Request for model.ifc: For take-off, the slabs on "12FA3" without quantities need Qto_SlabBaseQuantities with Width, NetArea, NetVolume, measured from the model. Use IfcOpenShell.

First a look at what the model holds.

```python
import ifcopenshell
import ifcopenshell.util.element
import ifcopenshell.util.unit

model = ifcopenshell.open("model.ifc")
print(model.schema)
for unit_type in ("LENGTHUNIT", "AREAUNIT", "VOLUMEUNIT"):
    print(unit_type, ifcopenshell.util.unit.calculate_unit_scale(model, unit_type))
storey = next(s for s in model.by_type("IfcBuildingStorey") if s.Name == "12FA3")
slabs = [e for e in ifcopenshell.util.element.get_decomposition(storey) if e.is_a("IfcSlab")]
for e in sorted(slabs, key=lambda e: e.id()):
    print(e.id(), e.is_a(), e.Name, list(ifcopenshell.util.element.get_psets(e, qtos_only=True)), sep=" | ")
```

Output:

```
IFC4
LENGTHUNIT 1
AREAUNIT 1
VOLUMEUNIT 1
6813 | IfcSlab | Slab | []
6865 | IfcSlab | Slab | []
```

```python
import ifcopenshell
import ifcopenshell.api.pset
import ifcopenshell.geom
import ifcopenshell.util.element
import ifcopenshell.util.shape
import ifcopenshell.util.unit

model = ifcopenshell.open("model.ifc")
unit_scale = ifcopenshell.util.unit.calculate_unit_scale(model)
area_scale = ifcopenshell.util.unit.calculate_unit_scale(model, "AREAUNIT")
volume_scale = ifcopenshell.util.unit.calculate_unit_scale(model, "VOLUMEUNIT")
settings = ifcopenshell.geom.settings()

storey = next(s for s in model.by_type("IfcBuildingStorey") if s.Name == "12FA3")
slabs = [e for e in ifcopenshell.util.element.get_decomposition(storey) if e.is_a("IfcSlab")]

for e in sorted(slabs, key=lambda e: e.id()):
    if ifcopenshell.util.element.get_psets(e, qtos_only=True, should_inherit=False):
        continue
    # Geometry comes back in metres, in the element's own axes.
    shape = ifcopenshell.geom.create_shape(settings, e)
    values = {
        "Width": ifcopenshell.util.shape.get_z(shape.geometry) / unit_scale,
        "NetArea": ifcopenshell.util.shape.get_footprint_area(shape.geometry) / area_scale,
        "NetVolume": ifcopenshell.util.shape.get_volume(shape.geometry) / volume_scale,
    }
    qto = ifcopenshell.api.pset.add_qto(model, product=e, name="Qto_SlabBaseQuantities")
    ifcopenshell.api.pset.edit_qto(model, qto=qto, properties=values)
    print(e.id(), {k: round(v, 3) for k, v in values.items()})

model.write("model_rev.ifc")
```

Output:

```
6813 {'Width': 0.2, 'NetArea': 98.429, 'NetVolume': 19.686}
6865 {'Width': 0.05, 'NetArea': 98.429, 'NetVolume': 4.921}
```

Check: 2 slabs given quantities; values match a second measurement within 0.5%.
